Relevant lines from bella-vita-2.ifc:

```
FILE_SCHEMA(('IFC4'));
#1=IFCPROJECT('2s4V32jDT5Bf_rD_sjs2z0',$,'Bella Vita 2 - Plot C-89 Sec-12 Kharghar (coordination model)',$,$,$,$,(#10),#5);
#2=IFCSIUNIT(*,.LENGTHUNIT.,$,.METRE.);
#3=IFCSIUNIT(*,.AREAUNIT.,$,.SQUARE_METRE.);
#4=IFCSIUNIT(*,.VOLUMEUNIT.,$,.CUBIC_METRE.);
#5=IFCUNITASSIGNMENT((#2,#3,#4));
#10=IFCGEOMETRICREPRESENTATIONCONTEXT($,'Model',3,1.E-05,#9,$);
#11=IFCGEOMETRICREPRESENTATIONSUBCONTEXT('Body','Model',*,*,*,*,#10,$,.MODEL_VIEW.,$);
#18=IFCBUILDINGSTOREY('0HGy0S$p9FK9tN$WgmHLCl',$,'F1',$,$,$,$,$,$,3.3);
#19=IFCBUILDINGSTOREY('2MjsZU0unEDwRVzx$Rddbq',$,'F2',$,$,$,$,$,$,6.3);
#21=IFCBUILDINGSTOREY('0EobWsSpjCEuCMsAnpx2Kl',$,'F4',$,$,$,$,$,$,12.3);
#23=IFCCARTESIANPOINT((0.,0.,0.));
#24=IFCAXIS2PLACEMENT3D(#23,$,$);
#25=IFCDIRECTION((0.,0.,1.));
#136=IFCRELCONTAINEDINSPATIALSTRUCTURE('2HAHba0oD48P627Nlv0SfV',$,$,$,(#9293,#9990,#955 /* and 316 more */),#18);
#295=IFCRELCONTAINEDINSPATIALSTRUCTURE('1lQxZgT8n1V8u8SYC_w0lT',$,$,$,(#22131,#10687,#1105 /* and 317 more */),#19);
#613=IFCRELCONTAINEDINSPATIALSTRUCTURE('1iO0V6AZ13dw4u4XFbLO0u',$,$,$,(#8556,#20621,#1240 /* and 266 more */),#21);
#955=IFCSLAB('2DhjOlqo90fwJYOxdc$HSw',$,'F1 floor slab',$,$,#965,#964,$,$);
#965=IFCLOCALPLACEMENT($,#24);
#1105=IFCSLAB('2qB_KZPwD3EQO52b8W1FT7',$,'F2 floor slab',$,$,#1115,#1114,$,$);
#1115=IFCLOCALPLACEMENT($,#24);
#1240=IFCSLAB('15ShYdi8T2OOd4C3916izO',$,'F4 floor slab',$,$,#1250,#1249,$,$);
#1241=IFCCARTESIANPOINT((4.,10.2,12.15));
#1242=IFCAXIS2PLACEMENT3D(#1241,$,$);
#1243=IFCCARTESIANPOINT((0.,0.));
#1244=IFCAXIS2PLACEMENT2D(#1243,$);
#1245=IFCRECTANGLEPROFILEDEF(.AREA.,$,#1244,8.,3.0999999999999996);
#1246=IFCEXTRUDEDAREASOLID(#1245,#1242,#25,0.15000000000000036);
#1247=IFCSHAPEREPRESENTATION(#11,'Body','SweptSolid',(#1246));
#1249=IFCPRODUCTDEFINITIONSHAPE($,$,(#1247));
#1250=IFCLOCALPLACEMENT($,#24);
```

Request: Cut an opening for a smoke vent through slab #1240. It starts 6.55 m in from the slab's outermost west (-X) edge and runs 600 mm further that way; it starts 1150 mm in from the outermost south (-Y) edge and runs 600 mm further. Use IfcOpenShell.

```python
import numpy as np
import ifcopenshell
import ifcopenshell.api.feature
import ifcopenshell.api.geometry
import ifcopenshell.api.root
import ifcopenshell.geom
import ifcopenshell.util.placement
import ifcopenshell.util.representation
import ifcopenshell.util.shape
import ifcopenshell.util.unit

model = ifcopenshell.open("bella-vita-2.ifc")
unit_scale = ifcopenshell.util.unit.calculate_unit_scale(model)
settings = ifcopenshell.geom.settings()


def volume(element):
    """Net volume in cubic metres, openings subtracted."""
    shape = ifcopenshell.geom.create_shape(settings, element)
    return ifcopenshell.util.shape.get_volume(shape.geometry)


slab = model.by_guid("15ShYdi8T2OOd4C3916izO")
before = volume(slab)

# Extent in the slab's own axes, in metres. The edges named are its -X and -Y sides.
slab_shape = ifcopenshell.geom.create_shape(settings, slab)
vertices = ifcopenshell.util.shape.get_vertices(slab_shape.geometry)
x_min, y_min, bottom = vertices.min(axis=0)
top = vertices[:, 2].max()

opening = ifcopenshell.api.root.create_entity(model, ifc_class="IfcOpeningElement", name="Smoke vent opening", predefined_type="OPENING")
context = ifcopenshell.util.representation.get_context(model, "Model", "Body", "MODEL_VIEW")
width, depth = 0.6, 0.6
outline = [(0.0, 0.0), (width, 0.0), (width, depth), (0.0, depth), (0.0, 0.0)]
# Overshoot both faces by 50 mm so the cut is clean.
shape = ifcopenshell.api.geometry.add_slab_representation(
    model, context=context, depth=top - bottom + 0.1, polyline=outline
)
ifcopenshell.api.geometry.assign_representation(model, product=opening, representation=shape)

matrix = ifcopenshell.util.placement.get_local_placement(slab.ObjectPlacement)
matrix[:, 3] = matrix @ np.append(np.array([x_min + 6.55, y_min + 1.15, bottom - 0.05]) / unit_scale, 1.0)
ifcopenshell.api.geometry.edit_object_placement(model, product=opening, matrix=matrix, is_si=False)
ifcopenshell.api.feature.add_feature(model, feature=opening, element=slab)

after = volume(slab)

print(f"slab volume {before:.3f} -> {after:.3f} m3")

model.write("bella-vita-2-out.ifc")
```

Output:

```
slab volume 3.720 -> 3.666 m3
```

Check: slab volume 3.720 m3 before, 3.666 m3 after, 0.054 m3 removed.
